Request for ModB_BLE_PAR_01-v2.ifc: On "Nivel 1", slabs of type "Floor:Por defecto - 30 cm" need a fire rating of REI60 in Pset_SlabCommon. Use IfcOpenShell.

First a look at what the model holds.

```python
import ifcopenshell
import ifcopenshell.util.element

model = ifcopenshell.open("ModB_BLE_PAR_01-v2.ifc")
print(model.schema)
storey = next(s for s in model.by_type("IfcBuildingStorey") if s.Name == "Nivel 1")
slabs = [e for e in ifcopenshell.util.element.get_decomposition(storey) if e.is_a("IfcSlab")]
seen = {}
for e in slabs:
    element_type = ifcopenshell.util.element.get_type(e)
    key = (element_type.Name if element_type != e and element_type else None, ifcopenshell.util.element.get_pset(e, "Pset_SlabCommon", "FireRating"))
    seen[key] = seen.get(key, 0) + 1
for (name, value), count in sorted(seen.items(), key=str):
    print(count, "x", name, "|", value)
```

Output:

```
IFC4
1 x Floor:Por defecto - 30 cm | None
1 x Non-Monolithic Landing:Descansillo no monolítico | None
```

```python
import ifcopenshell
import ifcopenshell.api.pset
import ifcopenshell.util.element

model = ifcopenshell.open("ModB_BLE_PAR_01-v2.ifc")

storey = next(s for s in model.by_type("IfcBuildingStorey") if s.Name == "Nivel 1")
slabs = [e for e in ifcopenshell.util.element.get_decomposition(storey) if e.is_a("IfcSlab")]

count = 0
for e in slabs:
    element_type = ifcopenshell.util.element.get_type(e)
    if element_type in (None, e) or element_type.Name != "Floor:Por defecto - 30 cm":
        continue
    # add_pset returns the element's existing set when there is one.
    pset = ifcopenshell.api.pset.add_pset(model, product=e, name="Pset_SlabCommon")
    ifcopenshell.api.pset.edit_pset(model, pset=pset, properties={"FireRating": "REI60"})
    count += 1

print(count, "slabs updated")

model.write("ModB_BLE_PAR_01-v2_updated.ifc")
```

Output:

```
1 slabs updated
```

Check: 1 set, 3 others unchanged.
